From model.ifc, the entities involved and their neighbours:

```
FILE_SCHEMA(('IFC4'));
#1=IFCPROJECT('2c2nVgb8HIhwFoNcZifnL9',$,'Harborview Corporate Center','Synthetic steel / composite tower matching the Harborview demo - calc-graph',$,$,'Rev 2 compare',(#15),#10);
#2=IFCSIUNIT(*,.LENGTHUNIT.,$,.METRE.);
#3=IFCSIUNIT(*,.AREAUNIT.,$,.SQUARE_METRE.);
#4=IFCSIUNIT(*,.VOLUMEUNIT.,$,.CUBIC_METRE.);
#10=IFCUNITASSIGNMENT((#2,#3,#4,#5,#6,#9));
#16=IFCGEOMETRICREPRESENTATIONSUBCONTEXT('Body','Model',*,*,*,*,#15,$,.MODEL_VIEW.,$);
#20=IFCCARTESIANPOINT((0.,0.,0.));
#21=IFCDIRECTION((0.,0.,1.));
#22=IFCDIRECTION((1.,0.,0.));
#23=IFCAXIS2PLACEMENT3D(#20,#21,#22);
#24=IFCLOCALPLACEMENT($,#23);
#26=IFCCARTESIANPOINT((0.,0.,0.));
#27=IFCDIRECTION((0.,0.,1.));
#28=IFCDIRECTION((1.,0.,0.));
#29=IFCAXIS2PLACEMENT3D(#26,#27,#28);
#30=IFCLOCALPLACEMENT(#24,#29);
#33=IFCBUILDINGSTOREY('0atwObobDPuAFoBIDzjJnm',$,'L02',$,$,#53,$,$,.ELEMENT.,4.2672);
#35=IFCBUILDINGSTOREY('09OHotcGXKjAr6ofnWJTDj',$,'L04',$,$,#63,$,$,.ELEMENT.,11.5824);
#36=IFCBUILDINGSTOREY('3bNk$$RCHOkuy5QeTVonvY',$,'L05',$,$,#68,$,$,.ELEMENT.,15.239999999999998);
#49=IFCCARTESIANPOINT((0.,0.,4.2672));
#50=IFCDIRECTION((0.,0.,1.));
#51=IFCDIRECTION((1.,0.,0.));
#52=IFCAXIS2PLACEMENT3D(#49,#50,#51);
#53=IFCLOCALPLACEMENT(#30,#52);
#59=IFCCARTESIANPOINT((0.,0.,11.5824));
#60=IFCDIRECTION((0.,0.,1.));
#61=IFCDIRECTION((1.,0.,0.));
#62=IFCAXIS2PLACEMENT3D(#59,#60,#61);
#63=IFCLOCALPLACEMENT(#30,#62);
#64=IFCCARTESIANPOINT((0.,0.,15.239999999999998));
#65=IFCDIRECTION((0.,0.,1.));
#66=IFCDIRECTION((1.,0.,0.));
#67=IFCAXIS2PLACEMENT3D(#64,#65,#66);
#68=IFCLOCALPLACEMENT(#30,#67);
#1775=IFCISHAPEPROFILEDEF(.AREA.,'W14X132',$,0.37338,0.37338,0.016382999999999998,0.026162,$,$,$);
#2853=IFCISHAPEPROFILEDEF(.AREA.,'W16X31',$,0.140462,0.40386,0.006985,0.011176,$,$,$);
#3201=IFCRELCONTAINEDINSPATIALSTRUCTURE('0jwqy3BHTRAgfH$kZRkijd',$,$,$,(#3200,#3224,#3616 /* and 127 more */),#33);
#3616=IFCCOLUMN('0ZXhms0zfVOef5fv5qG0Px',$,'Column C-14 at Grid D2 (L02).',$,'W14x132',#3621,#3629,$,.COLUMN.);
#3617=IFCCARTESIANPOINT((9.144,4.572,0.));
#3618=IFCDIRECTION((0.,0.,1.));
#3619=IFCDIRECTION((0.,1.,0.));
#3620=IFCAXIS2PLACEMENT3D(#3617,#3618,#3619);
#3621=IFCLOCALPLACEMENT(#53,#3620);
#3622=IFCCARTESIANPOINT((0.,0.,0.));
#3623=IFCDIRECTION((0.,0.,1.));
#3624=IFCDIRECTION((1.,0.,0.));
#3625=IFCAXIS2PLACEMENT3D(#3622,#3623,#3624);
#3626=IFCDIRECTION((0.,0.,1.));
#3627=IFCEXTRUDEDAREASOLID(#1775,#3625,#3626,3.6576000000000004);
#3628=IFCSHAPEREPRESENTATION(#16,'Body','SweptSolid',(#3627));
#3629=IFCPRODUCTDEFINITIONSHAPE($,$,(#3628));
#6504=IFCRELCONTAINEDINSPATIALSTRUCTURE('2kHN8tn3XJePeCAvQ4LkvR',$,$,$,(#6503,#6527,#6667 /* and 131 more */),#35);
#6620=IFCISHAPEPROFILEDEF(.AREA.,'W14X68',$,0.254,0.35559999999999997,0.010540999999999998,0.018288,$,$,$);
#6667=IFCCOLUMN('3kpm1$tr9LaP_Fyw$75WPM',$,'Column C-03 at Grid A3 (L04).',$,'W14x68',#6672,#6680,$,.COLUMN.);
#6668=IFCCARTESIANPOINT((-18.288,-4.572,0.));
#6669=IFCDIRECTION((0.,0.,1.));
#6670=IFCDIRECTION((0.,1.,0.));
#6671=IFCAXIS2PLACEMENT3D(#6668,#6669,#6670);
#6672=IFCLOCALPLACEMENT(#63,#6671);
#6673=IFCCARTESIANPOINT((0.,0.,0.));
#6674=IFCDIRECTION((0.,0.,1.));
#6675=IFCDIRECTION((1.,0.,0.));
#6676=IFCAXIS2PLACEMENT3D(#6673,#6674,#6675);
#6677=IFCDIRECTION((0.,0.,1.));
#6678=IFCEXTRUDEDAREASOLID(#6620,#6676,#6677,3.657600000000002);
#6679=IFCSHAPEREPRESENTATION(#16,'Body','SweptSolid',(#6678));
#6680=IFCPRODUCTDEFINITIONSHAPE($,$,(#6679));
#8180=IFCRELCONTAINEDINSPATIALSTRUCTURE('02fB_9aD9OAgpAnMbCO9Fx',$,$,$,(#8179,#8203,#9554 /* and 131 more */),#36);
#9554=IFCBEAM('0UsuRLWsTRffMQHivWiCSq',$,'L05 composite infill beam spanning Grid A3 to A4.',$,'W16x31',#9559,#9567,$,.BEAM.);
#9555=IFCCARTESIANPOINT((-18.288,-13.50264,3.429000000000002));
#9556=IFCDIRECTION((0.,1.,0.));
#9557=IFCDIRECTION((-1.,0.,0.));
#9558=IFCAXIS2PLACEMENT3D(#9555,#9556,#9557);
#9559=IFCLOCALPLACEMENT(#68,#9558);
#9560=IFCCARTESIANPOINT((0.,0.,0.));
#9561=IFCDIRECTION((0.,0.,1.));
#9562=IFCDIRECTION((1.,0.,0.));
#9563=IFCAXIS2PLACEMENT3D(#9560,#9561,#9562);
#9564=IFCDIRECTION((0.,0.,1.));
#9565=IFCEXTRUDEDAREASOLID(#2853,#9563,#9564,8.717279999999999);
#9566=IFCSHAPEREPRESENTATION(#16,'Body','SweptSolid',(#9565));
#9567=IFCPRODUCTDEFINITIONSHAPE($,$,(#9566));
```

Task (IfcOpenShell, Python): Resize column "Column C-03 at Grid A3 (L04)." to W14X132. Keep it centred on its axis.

```python
import ifcopenshell
import ifcopenshell.util.element
import ifcopenshell.util.representation

model = ifcopenshell.open("model.ifc")

member = model.by_id(6667)
source = next(p for p in model.by_type("IfcIShapeProfileDef") if p.ProfileName == "W14X132")

body = ifcopenshell.util.representation.get_representation(member, "Model", "Body")
solid = body.Items[0]
old_profile = solid.SweptArea

# Copy the section's sizes but keep this member's own profile position.
profile = ifcopenshell.util.element.copy(model, source)
profile.Position = old_profile.Position
solid.SweptArea = profile
if not model.get_total_inverses(old_profile):
    ifcopenshell.util.element.remove_deep2(model, old_profile)

print(solid.SweptArea)

model.write("model_edited.ifc")
```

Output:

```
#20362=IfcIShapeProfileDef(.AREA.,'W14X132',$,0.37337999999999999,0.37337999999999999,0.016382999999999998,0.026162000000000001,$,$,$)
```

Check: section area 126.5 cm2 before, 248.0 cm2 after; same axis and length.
